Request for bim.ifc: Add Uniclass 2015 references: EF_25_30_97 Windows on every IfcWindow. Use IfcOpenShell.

First a look at what the model holds.

```python
import ifcopenshell

model = ifcopenshell.open("bim.ifc")
print(model.schema)
print("classifications:", [c.Name for c in model.by_type("IfcClassification")])
for ifc_class in ("IfcDoor", "IfcRoof", "IfcStair", "IfcWall", "IfcWindow"):
    print(ifc_class, len(model.by_type(ifc_class)))
```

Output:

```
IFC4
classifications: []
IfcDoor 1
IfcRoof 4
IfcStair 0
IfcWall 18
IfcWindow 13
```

```python
import ifcopenshell
import ifcopenshell.api.classification

model = ifcopenshell.open("bim.ifc")

system = ifcopenshell.api.classification.add_classification(model, classification="Uniclass 2015")

codes = {
    "IfcWindow": ("EF_25_30_97", "Windows"),
}
for ifc_class, (code, name) in codes.items():
    products = model.by_type(ifc_class)
    ifcopenshell.api.classification.add_reference(
        model, products=products, classification=system, identification=code, name=name
    )
    print(code, len(products))

model.write("bim_edited.ifc")
```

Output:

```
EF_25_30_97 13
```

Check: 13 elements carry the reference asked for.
